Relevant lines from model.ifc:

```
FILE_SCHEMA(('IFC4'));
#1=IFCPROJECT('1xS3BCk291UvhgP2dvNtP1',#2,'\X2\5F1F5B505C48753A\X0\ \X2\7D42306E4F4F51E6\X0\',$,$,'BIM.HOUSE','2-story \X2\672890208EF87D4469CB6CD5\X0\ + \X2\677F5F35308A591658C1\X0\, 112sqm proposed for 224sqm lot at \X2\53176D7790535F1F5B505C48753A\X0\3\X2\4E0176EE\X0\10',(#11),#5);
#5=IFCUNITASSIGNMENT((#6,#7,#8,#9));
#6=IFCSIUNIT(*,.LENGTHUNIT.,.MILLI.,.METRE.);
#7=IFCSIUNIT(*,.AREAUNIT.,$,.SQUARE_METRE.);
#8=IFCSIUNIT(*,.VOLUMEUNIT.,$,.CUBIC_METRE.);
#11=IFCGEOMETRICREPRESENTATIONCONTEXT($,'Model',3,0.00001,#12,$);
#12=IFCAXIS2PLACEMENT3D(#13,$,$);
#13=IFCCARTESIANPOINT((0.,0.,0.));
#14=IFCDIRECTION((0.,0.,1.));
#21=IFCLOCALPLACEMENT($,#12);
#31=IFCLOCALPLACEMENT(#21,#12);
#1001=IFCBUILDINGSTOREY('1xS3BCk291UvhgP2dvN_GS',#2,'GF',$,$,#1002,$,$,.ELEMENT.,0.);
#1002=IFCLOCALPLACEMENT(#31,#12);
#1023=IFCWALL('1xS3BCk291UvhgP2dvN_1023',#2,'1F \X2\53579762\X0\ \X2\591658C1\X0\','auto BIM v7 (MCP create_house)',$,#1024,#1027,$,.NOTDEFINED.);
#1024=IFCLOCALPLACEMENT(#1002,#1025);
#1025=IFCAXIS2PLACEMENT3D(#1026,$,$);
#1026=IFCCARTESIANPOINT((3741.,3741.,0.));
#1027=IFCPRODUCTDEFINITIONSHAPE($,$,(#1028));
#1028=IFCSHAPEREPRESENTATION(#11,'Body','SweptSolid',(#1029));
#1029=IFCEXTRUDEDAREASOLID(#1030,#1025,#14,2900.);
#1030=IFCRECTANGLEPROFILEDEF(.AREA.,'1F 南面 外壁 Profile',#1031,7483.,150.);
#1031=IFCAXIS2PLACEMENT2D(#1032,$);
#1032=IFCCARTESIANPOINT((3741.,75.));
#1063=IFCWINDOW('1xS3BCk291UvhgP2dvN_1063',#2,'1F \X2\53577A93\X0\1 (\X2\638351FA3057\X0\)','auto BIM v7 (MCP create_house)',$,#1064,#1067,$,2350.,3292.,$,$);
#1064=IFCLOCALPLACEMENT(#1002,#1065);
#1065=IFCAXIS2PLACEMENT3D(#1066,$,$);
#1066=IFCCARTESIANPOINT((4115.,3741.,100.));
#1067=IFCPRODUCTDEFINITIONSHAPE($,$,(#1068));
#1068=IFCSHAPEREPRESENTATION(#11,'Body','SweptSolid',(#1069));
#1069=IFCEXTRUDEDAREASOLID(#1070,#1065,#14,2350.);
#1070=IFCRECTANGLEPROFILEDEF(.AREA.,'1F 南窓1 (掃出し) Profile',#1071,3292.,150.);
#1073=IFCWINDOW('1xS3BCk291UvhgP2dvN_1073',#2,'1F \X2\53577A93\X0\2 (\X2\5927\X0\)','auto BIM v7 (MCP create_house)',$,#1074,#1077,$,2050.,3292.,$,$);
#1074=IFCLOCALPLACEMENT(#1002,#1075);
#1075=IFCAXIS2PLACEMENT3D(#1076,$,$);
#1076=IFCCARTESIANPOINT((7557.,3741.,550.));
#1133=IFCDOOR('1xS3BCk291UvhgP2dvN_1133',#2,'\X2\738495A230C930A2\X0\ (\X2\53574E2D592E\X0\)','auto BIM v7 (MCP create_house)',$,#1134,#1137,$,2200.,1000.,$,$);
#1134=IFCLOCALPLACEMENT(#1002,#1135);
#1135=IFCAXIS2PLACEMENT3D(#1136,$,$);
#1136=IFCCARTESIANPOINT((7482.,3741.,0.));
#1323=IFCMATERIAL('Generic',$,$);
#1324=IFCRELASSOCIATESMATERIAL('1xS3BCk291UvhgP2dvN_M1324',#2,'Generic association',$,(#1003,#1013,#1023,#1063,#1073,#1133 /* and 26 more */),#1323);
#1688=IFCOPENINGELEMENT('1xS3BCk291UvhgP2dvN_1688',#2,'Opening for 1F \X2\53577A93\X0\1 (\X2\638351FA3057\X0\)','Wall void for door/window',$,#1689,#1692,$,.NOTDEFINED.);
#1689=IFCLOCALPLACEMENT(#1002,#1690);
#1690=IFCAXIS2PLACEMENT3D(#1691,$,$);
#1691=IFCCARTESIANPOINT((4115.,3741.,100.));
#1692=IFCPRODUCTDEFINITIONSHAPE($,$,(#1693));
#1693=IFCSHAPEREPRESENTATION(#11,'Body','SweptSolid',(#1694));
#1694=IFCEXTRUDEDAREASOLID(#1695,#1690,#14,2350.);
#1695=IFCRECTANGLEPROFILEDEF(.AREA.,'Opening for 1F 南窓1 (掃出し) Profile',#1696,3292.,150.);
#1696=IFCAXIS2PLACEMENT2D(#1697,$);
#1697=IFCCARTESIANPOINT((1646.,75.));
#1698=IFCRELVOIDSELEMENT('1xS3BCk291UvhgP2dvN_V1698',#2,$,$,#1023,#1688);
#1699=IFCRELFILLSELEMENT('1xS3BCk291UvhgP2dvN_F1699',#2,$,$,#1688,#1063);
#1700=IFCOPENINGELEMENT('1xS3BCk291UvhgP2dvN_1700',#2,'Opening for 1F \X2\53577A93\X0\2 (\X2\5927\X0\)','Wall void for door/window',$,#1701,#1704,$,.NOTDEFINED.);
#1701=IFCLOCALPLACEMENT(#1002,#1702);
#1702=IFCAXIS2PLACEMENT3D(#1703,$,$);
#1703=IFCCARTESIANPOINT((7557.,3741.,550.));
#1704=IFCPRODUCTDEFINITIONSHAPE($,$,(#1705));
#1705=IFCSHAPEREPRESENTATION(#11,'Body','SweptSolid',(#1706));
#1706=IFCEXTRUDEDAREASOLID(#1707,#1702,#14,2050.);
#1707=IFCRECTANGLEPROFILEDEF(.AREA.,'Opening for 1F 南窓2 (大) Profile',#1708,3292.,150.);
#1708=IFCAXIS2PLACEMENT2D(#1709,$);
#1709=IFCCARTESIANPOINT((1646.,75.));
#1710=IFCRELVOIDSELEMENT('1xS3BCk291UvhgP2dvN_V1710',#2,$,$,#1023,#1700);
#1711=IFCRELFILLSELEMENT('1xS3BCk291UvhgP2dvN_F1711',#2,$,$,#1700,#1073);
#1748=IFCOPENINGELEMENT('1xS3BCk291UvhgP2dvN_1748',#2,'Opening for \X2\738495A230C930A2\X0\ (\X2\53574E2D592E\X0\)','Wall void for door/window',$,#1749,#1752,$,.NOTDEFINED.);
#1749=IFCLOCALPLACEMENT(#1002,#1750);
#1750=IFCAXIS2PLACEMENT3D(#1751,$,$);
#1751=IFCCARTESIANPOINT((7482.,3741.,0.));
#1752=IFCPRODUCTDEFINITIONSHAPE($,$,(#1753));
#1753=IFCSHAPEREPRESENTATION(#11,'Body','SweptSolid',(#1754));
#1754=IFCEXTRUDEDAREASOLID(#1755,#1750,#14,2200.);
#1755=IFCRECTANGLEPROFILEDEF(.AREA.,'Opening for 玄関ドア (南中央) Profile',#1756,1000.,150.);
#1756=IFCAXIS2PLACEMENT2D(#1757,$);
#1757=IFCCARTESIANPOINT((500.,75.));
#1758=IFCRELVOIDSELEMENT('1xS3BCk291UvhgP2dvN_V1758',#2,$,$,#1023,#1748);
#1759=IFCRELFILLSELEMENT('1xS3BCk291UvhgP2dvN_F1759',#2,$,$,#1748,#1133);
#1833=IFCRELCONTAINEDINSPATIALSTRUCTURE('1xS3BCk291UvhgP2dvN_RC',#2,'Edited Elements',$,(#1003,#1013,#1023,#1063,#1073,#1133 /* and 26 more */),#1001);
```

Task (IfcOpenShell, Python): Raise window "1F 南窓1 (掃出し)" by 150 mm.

```python
import numpy as np
import ifcopenshell
import ifcopenshell.api.geometry
import ifcopenshell.util.placement
import ifcopenshell.util.unit

model = ifcopenshell.open("model.ifc")
unit_scale = ifcopenshell.util.unit.calculate_unit_scale(model)

window = model.by_guid("1xS3BCk291UvhgP2dvN_1063")
opening = window.FillsVoids[0].RelatingOpeningElement
dz = 0.15 / unit_scale

shift = np.array([0.0, 0.0, dz])
# The window is not placed relative to its opening, so move both.
for product in (opening, window):
    matrix = ifcopenshell.util.placement.get_local_placement(product.ObjectPlacement)
    matrix[:3, 3] += shift
    ifcopenshell.api.geometry.edit_object_placement(model, product=product, matrix=matrix, is_si=False)

print(f"moved by {dz * unit_scale:+.3f} m")

model.write("model_edited.ifc")
```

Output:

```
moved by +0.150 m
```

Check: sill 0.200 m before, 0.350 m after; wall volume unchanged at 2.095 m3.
